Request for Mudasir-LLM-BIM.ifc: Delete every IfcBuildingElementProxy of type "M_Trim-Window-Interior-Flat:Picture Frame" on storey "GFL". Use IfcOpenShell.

First a look at what the model holds.

```python
import ifcopenshell
import ifcopenshell.util.element

model = ifcopenshell.open("Mudasir-LLM-BIM.ifc")
print(model.schema)
storey = next(s for s in model.by_type("IfcBuildingStorey") if s.Name == "GFL")
proxies = [e for e in ifcopenshell.util.element.get_decomposition(storey) if e.is_a("IfcBuildingElementProxy")]
seen = {}
for e in proxies:
    element_type = ifcopenshell.util.element.get_type(e)
    name = element_type.Name if element_type not in (None, e) else None
    seen[name] = seen.get(name, 0) + 1
for name, count in sorted(seen.items(), key=str):
    print(count, "x", name)
```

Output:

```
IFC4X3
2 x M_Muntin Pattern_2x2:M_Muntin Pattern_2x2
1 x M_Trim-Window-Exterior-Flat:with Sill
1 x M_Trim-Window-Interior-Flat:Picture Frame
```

```python
import ifcopenshell
import ifcopenshell.api.root
import ifcopenshell.util.element

model = ifcopenshell.open("Mudasir-LLM-BIM.ifc")

storey = next(s for s in model.by_type("IfcBuildingStorey") if s.Name == "GFL")
proxies = [e for e in ifcopenshell.util.element.get_decomposition(storey) if e.is_a("IfcBuildingElementProxy")]
targets = [e for e in proxies if (t := ifcopenshell.util.element.get_type(e)) not in (None, e) and t.Name == "M_Trim-Window-Interior-Flat:Picture Frame"]

for e in targets:
    ifcopenshell.api.root.remove_product(model, product=e)
print(len(targets), "removed")

model.write("Mudasir-LLM-BIM-out.ifc")
```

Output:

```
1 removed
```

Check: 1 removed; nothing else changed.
